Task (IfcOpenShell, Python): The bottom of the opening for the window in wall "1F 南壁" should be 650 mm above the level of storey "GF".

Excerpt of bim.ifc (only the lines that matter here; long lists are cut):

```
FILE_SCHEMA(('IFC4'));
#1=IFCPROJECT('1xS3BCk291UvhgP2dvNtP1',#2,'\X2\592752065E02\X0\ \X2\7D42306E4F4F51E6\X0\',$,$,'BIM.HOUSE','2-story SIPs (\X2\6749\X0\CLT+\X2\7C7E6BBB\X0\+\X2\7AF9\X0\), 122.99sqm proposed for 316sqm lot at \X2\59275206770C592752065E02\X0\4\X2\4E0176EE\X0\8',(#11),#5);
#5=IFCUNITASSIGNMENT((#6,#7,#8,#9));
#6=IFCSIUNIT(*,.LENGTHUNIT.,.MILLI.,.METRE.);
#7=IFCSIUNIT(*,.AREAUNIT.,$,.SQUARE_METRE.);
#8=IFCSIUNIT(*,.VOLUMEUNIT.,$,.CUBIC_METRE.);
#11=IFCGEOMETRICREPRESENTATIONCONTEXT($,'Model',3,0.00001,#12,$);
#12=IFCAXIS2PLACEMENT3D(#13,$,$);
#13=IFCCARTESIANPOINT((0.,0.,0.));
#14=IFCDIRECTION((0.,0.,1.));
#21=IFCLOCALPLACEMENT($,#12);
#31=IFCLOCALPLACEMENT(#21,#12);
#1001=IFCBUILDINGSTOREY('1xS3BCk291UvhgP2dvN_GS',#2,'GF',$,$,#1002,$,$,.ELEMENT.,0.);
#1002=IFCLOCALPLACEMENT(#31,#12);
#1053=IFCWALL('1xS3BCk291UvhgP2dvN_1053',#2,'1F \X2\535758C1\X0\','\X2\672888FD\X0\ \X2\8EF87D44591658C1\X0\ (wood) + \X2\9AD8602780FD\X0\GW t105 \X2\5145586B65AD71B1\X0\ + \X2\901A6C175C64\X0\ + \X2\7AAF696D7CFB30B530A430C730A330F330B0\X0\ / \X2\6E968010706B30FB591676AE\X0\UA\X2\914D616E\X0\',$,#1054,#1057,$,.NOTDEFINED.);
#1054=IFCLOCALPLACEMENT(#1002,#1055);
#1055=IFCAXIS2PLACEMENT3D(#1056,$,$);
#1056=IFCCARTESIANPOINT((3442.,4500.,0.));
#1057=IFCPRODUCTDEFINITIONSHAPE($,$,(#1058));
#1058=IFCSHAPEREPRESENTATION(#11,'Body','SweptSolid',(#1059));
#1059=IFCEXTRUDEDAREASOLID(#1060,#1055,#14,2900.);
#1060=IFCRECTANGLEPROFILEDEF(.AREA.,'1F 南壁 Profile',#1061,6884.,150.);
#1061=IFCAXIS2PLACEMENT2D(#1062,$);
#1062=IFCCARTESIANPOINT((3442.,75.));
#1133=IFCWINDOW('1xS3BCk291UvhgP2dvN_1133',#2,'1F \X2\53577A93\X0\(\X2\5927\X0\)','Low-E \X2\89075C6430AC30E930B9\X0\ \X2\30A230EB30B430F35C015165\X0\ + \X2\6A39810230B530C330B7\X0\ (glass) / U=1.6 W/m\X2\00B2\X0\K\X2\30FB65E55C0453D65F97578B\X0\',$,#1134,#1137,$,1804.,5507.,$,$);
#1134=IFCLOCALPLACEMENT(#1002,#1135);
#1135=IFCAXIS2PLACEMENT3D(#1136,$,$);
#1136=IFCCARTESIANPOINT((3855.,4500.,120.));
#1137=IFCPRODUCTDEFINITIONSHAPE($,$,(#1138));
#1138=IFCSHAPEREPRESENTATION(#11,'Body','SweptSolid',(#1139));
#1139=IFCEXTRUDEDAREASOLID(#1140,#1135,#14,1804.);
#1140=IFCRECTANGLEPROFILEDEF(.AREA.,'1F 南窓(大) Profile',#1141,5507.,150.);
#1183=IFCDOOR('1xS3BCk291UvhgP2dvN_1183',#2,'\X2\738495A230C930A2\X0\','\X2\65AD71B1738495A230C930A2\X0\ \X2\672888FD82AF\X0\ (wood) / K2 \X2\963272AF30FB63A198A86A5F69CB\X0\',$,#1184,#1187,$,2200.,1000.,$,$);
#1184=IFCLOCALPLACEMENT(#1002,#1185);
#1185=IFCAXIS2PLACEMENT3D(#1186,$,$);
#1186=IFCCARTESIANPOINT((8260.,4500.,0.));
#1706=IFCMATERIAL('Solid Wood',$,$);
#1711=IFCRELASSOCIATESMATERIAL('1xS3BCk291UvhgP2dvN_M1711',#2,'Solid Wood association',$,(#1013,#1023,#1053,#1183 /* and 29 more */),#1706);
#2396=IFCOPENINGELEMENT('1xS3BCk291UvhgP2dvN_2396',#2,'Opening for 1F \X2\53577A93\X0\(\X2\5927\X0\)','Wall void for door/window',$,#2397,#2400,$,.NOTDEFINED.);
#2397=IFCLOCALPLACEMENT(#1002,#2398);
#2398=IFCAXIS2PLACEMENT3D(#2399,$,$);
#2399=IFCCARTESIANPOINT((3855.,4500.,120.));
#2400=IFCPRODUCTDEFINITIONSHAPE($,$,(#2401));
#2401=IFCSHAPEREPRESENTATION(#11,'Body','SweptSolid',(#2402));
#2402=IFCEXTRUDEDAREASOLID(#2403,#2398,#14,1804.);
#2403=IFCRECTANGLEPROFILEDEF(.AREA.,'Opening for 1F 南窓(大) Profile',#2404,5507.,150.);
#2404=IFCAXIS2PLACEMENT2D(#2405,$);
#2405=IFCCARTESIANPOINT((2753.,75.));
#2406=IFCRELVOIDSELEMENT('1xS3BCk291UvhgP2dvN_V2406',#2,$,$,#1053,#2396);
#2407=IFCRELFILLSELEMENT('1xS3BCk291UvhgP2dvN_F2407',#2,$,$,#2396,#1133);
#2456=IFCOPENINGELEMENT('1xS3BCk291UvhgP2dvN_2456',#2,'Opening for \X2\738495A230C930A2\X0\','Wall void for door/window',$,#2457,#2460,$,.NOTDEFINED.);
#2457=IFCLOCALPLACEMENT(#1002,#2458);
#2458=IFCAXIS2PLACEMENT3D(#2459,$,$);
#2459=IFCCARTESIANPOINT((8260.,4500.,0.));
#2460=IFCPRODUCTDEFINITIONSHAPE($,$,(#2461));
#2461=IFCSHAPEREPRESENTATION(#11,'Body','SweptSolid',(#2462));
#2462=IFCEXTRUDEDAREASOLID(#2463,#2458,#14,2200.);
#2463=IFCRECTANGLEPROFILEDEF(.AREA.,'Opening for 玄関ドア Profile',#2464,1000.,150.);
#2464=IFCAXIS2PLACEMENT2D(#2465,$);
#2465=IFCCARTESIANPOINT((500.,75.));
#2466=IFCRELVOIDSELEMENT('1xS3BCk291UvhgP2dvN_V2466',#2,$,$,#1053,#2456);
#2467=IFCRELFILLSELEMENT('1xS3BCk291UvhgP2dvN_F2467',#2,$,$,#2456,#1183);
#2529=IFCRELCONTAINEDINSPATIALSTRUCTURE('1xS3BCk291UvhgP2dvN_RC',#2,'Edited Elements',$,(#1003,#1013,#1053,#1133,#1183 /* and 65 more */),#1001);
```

```python
import numpy as np
import ifcopenshell
import ifcopenshell.api.geometry
import ifcopenshell.geom
import ifcopenshell.util.element
import ifcopenshell.util.placement
import ifcopenshell.util.shape
import ifcopenshell.util.unit

model = ifcopenshell.open("bim.ifc")
unit_scale = ifcopenshell.util.unit.calculate_unit_scale(model)

window = model.by_guid("1xS3BCk291UvhgP2dvN_1133")
opening = window.FillsVoids[0].RelatingOpeningElement
storey = ifcopenshell.util.element.get_container(window, ifc_class="IfcBuildingStorey")
level = ifcopenshell.util.placement.get_local_placement(storey.ObjectPlacement)[2, 3]

# The opening's origin need not be at the sill, so measure its lowest point.
shape = ifcopenshell.geom.create_shape(ifcopenshell.geom.settings(), opening)
bottom = ifcopenshell.util.shape.get_shape_bottom_elevation(shape, shape.geometry) / unit_scale
dz = level + 650.0 - bottom

shift = np.array([0.0, 0.0, dz])
# The window is not placed relative to its opening, so move both.
for product in (opening, window):
    matrix = ifcopenshell.util.placement.get_local_placement(product.ObjectPlacement)
    matrix[:3, 3] += shift
    ifcopenshell.api.geometry.edit_object_placement(model, product=product, matrix=matrix, is_si=False)

print(f"moved by {dz * unit_scale:+.3f} m")

model.write("bim-out.ifc")
```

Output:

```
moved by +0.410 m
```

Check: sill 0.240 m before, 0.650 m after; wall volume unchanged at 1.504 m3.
